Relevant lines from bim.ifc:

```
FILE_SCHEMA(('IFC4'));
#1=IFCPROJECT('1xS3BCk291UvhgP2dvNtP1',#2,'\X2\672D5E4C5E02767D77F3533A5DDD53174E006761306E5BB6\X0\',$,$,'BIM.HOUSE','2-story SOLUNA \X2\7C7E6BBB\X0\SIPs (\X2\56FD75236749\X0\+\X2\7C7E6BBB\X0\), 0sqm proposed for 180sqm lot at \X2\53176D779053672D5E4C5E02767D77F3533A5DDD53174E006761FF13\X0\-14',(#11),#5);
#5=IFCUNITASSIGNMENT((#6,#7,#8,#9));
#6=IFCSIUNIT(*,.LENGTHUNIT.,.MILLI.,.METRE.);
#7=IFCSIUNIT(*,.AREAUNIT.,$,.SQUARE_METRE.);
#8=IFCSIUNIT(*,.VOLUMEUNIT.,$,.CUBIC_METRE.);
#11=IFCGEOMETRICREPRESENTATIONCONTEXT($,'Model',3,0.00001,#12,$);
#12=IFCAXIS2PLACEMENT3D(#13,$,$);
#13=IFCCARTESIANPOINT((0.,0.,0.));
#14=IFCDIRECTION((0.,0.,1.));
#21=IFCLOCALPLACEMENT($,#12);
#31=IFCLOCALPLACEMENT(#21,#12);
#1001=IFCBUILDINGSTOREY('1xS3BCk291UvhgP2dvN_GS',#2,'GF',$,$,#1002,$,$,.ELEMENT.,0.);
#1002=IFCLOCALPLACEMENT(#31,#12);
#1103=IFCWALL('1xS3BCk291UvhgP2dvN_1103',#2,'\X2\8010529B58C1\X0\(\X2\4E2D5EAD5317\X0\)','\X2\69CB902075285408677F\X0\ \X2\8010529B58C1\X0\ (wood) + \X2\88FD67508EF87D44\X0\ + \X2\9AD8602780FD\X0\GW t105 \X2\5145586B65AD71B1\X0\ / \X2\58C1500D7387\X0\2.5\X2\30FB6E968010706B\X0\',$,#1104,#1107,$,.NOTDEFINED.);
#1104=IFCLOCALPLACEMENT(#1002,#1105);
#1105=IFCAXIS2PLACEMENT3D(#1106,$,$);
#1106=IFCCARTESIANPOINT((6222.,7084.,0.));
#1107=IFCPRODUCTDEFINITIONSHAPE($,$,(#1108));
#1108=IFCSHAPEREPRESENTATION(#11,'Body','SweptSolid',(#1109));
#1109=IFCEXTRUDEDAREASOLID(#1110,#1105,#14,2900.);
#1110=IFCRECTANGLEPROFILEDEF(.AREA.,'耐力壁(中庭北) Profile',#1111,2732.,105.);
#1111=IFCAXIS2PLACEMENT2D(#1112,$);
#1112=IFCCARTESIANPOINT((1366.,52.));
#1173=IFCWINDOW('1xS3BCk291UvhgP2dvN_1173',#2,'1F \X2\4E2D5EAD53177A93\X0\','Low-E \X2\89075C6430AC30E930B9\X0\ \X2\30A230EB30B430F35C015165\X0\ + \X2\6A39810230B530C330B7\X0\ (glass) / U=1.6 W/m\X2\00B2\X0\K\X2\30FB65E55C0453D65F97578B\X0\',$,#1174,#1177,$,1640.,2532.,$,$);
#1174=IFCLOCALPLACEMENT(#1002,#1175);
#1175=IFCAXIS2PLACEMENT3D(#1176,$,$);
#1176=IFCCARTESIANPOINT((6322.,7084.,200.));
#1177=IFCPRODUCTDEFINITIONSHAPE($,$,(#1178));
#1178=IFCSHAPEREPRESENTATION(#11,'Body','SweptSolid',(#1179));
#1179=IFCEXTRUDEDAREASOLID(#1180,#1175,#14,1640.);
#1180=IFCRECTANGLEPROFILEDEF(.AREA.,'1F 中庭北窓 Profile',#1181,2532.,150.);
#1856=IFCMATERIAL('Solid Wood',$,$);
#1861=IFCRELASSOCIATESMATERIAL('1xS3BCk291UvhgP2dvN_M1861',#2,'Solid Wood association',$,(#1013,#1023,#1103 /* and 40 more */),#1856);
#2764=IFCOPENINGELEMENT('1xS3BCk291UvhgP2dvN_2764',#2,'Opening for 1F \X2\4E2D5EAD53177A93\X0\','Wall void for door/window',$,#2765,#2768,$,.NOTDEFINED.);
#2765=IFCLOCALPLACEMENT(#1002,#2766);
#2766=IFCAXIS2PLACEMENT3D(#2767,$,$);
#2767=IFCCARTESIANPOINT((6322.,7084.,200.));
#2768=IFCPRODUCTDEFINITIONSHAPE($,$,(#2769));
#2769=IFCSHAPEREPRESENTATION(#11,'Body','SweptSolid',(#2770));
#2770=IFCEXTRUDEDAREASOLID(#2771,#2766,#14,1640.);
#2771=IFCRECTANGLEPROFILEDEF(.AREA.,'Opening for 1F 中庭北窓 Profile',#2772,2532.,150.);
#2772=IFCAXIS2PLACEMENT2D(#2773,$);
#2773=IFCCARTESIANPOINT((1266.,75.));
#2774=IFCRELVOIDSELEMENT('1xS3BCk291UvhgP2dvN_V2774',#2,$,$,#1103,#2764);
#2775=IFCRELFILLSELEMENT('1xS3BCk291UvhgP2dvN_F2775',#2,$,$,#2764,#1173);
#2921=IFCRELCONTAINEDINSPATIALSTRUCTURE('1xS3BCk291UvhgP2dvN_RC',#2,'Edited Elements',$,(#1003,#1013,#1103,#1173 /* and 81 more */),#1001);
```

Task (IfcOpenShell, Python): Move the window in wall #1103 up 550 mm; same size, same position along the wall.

```python
import numpy as np
import ifcopenshell
import ifcopenshell.api.geometry
import ifcopenshell.util.placement
import ifcopenshell.util.unit

model = ifcopenshell.open("bim.ifc")
unit_scale = ifcopenshell.util.unit.calculate_unit_scale(model)

window = model.by_guid("1xS3BCk291UvhgP2dvN_1173")
opening = window.FillsVoids[0].RelatingOpeningElement
dz = 0.55 / unit_scale

shift = np.array([0.0, 0.0, dz])
# The window is not placed relative to its opening, so move both.
for product in (opening, window):
    matrix = ifcopenshell.util.placement.get_local_placement(product.ObjectPlacement)
    matrix[:3, 3] += shift
    ifcopenshell.api.geometry.edit_object_placement(model, product=product, matrix=matrix, is_si=False)

print(f"moved by {dz * unit_scale:+.3f} m")

model.write("bim-out.ifc")
```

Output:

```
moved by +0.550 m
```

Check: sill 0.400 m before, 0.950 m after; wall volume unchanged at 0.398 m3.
